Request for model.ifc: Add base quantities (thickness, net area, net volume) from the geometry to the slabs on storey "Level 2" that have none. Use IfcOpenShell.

First a look at what the model holds.

```python
import ifcopenshell
import ifcopenshell.util.element
import ifcopenshell.util.unit

model = ifcopenshell.open("model.ifc")
print(model.schema)
for unit_type in ("LENGTHUNIT", "AREAUNIT", "VOLUMEUNIT"):
    print(unit_type, ifcopenshell.util.unit.calculate_unit_scale(model, unit_type))
storey = next(s for s in model.by_type("IfcBuildingStorey") if s.Name == "Level 2")
slabs = [e for e in ifcopenshell.util.element.get_decomposition(storey) if e.is_a("IfcSlab")]
for e in sorted(slabs, key=lambda e: e.id()):
    print(e.id(), e.is_a(), e.Name, list(ifcopenshell.util.element.get_psets(e, qtos_only=True)), sep=" | ")
```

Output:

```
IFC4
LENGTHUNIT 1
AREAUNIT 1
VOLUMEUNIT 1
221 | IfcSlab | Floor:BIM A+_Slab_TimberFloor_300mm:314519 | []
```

```python
import ifcopenshell
import ifcopenshell.api.pset
import ifcopenshell.geom
import ifcopenshell.util.element
import ifcopenshell.util.shape
import ifcopenshell.util.unit

model = ifcopenshell.open("model.ifc")
unit_scale = ifcopenshell.util.unit.calculate_unit_scale(model)
area_scale = ifcopenshell.util.unit.calculate_unit_scale(model, "AREAUNIT")
volume_scale = ifcopenshell.util.unit.calculate_unit_scale(model, "VOLUMEUNIT")
settings = ifcopenshell.geom.settings()

storey = next(s for s in model.by_type("IfcBuildingStorey") if s.Name == "Level 2")
slabs = [e for e in ifcopenshell.util.element.get_decomposition(storey) if e.is_a("IfcSlab")]

for e in sorted(slabs, key=lambda e: e.id()):
    if ifcopenshell.util.element.get_psets(e, qtos_only=True, should_inherit=False):
        continue
    # Geometry comes back in metres, in the element's own axes.
    shape = ifcopenshell.geom.create_shape(settings, e)
    values = {
        "Width": ifcopenshell.util.shape.get_z(shape.geometry) / unit_scale,
        "NetArea": ifcopenshell.util.shape.get_footprint_area(shape.geometry) / area_scale,
        "NetVolume": ifcopenshell.util.shape.get_volume(shape.geometry) / volume_scale,
    }
    qto = ifcopenshell.api.pset.add_qto(model, product=e, name="Qto_SlabBaseQuantities")
    ifcopenshell.api.pset.edit_qto(model, qto=qto, properties=values)
    print(e.id(), {k: round(v, 3) for k, v in values.items()})

model.write("model_rev.ifc")
```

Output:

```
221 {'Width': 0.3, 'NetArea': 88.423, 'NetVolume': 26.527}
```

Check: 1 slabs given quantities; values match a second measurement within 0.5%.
